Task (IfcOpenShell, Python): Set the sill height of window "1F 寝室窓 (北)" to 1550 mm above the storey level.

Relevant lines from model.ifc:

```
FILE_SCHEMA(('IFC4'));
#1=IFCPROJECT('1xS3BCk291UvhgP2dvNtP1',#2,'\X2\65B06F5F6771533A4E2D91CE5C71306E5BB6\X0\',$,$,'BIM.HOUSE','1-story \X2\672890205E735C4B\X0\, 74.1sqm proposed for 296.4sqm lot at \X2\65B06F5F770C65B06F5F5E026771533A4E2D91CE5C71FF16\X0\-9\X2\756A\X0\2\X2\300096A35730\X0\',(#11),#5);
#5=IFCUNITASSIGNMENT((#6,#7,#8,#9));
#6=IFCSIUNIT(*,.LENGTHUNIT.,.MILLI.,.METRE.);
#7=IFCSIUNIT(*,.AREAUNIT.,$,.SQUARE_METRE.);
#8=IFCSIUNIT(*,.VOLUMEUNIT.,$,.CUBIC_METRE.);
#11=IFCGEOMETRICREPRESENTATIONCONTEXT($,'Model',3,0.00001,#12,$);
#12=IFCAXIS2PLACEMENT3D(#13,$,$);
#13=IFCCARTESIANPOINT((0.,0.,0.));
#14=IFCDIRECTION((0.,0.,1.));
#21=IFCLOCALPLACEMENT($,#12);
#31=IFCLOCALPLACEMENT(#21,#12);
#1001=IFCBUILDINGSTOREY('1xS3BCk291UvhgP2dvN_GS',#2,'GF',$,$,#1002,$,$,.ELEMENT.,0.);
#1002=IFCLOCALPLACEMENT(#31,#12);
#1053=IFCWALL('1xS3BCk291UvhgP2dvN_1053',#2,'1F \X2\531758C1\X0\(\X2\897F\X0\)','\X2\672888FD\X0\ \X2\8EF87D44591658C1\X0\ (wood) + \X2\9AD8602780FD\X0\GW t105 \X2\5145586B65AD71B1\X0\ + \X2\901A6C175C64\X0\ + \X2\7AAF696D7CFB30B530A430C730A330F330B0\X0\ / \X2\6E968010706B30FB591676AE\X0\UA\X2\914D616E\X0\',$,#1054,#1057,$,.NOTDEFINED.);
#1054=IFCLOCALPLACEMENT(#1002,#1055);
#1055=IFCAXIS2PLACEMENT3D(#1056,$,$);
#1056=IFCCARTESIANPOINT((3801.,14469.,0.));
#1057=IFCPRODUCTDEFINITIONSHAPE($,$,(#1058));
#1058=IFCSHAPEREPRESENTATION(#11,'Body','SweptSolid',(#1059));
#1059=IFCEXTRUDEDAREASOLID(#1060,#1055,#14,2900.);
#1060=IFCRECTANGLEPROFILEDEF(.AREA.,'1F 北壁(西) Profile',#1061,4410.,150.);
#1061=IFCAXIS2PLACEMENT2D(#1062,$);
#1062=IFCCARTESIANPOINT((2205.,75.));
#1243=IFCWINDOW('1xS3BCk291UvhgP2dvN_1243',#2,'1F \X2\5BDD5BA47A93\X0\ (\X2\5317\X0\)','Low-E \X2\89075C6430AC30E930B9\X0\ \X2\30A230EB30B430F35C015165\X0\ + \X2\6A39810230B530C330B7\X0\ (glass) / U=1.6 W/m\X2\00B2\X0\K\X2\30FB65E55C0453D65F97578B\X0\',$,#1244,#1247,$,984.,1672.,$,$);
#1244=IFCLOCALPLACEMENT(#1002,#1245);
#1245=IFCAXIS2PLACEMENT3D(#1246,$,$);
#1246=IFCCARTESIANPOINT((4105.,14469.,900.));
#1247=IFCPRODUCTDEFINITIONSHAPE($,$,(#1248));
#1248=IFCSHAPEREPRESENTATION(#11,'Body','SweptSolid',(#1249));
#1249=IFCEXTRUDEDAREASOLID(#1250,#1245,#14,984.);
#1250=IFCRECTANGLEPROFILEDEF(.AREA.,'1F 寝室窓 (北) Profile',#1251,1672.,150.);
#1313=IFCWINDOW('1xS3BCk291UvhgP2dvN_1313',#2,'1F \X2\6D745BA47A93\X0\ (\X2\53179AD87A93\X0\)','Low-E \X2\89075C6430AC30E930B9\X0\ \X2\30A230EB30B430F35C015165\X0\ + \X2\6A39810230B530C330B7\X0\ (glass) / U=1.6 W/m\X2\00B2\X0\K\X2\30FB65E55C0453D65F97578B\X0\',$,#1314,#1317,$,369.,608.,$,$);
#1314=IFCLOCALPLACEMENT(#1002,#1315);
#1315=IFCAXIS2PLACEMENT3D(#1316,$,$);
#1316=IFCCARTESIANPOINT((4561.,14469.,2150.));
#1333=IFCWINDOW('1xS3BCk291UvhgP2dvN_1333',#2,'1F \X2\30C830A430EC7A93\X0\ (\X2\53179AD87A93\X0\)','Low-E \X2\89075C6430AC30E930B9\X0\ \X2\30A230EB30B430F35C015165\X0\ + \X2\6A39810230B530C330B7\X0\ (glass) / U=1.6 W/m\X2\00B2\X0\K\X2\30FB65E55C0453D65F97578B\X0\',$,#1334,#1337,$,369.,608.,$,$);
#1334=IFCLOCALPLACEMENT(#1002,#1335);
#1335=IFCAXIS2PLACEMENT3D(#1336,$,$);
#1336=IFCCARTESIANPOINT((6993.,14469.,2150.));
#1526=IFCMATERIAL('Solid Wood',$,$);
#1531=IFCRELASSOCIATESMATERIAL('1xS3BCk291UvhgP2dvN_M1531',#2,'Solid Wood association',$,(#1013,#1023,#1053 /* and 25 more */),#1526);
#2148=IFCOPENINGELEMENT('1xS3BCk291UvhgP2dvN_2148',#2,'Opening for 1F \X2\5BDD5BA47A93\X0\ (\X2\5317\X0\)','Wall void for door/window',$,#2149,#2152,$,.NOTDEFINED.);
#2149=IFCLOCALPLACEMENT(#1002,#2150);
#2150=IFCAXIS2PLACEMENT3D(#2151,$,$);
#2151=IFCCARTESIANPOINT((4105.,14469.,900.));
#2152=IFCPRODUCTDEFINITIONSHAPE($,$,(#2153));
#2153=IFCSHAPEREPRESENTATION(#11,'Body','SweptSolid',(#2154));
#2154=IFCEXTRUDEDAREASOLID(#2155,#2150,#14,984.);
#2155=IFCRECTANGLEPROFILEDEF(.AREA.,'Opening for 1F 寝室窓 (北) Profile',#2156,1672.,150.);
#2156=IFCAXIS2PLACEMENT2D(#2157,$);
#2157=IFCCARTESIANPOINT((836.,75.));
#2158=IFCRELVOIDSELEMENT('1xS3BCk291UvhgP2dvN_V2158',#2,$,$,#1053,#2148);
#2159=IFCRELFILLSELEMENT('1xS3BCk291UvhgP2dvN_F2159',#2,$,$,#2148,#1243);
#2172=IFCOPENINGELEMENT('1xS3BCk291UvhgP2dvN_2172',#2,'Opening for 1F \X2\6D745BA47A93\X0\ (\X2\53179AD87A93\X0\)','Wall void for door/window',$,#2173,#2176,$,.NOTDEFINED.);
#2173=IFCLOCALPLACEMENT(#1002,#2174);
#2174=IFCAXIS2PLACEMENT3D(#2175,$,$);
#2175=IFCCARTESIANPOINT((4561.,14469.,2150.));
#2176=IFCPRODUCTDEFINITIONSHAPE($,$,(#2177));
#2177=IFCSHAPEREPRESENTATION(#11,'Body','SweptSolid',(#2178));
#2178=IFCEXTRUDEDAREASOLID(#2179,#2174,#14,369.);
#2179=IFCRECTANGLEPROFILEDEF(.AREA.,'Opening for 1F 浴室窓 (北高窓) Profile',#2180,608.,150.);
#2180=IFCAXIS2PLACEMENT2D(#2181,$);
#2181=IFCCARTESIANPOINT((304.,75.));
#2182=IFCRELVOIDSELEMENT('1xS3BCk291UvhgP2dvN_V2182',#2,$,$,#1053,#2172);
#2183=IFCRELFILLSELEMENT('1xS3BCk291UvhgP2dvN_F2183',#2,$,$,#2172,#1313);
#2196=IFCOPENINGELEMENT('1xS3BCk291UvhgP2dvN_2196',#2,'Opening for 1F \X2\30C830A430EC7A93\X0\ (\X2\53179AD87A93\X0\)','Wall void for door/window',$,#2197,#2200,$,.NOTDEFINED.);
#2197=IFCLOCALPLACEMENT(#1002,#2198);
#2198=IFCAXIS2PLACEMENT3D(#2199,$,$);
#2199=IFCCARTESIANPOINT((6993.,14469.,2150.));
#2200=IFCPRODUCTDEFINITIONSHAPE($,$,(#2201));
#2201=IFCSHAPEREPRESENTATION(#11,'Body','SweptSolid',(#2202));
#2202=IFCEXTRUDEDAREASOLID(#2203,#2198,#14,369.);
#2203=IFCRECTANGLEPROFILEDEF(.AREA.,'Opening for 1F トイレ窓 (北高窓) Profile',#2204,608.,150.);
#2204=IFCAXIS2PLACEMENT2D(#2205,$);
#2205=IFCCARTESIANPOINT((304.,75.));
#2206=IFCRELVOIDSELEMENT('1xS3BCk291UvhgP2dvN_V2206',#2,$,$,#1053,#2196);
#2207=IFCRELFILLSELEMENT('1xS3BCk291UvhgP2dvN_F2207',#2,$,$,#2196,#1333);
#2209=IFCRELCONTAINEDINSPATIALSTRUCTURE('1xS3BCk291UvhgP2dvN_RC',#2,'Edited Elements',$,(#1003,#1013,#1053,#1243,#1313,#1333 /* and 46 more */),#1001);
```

```python
import numpy as np
import ifcopenshell
import ifcopenshell.api.geometry
import ifcopenshell.geom
import ifcopenshell.util.element
import ifcopenshell.util.placement
import ifcopenshell.util.shape
import ifcopenshell.util.unit

model = ifcopenshell.open("model.ifc")
unit_scale = ifcopenshell.util.unit.calculate_unit_scale(model)

window = model.by_guid("1xS3BCk291UvhgP2dvN_1243")
opening = window.FillsVoids[0].RelatingOpeningElement
storey = ifcopenshell.util.element.get_container(window, ifc_class="IfcBuildingStorey")
level = ifcopenshell.util.placement.get_local_placement(storey.ObjectPlacement)[2, 3]

# The opening's origin need not be at the sill, so measure its lowest point.
shape = ifcopenshell.geom.create_shape(ifcopenshell.geom.settings(), opening)
bottom = ifcopenshell.util.shape.get_shape_bottom_elevation(shape, shape.geometry) / unit_scale
dz = level + 1.55 / unit_scale - bottom

shift = np.array([0.0, 0.0, dz])
# The window is not placed relative to its opening, so move both.
for product in (opening, window):
    matrix = ifcopenshell.util.placement.get_local_placement(product.ObjectPlacement)
    matrix[:3, 3] += shift
    ifcopenshell.api.geometry.edit_object_placement(model, product=product, matrix=matrix, is_si=False)

print(f"moved by {dz * unit_scale:+.3f} m")

model.write("model_updated.ifc")
```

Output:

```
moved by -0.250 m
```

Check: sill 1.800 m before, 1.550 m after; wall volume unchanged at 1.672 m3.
